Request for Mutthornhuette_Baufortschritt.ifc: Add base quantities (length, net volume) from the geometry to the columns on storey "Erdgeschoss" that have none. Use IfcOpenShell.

First a look at what the model holds.

```python
import ifcopenshell
import ifcopenshell.util.element
import ifcopenshell.util.unit

model = ifcopenshell.open("Mutthornhuette_Baufortschritt.ifc")
print(model.schema)
for unit_type in ("LENGTHUNIT", "AREAUNIT", "VOLUMEUNIT"):
    print(unit_type, ifcopenshell.util.unit.calculate_unit_scale(model, unit_type))
storey = next(s for s in model.by_type("IfcBuildingStorey") if s.Name == "Erdgeschoss")
columns = [e for e in ifcopenshell.util.element.get_decomposition(storey) if e.is_a("IfcColumn")]
for e in sorted(columns, key=lambda e: e.id()):
    print(e.id(), e.is_a(), e.Name, list(ifcopenshell.util.element.get_psets(e, qtos_only=True)), sep=" | ")
```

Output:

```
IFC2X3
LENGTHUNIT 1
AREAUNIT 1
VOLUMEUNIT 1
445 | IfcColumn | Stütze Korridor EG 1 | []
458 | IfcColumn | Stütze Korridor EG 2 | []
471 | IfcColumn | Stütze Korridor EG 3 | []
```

```python
import ifcopenshell
import ifcopenshell.api.pset
import ifcopenshell.geom
import ifcopenshell.util.element
import ifcopenshell.util.shape
import ifcopenshell.util.unit

model = ifcopenshell.open("Mutthornhuette_Baufortschritt.ifc")
unit_scale = ifcopenshell.util.unit.calculate_unit_scale(model)
volume_scale = ifcopenshell.util.unit.calculate_unit_scale(model, "VOLUMEUNIT")
settings = ifcopenshell.geom.settings()

storey = next(s for s in model.by_type("IfcBuildingStorey") if s.Name == "Erdgeschoss")
columns = [e for e in ifcopenshell.util.element.get_decomposition(storey) if e.is_a("IfcColumn")]

for e in sorted(columns, key=lambda e: e.id()):
    if ifcopenshell.util.element.get_psets(e, qtos_only=True, should_inherit=False):
        continue
    # Geometry comes back in metres, in the element's own axes.
    shape = ifcopenshell.geom.create_shape(settings, e)
    values = {
        "Length": ifcopenshell.util.shape.get_z(shape.geometry) / unit_scale,
        "NetVolume": ifcopenshell.util.shape.get_volume(shape.geometry) / volume_scale,
    }
    qto = ifcopenshell.api.pset.add_qto(model, product=e, name="BaseQuantities")
    ifcopenshell.api.pset.edit_qto(model, qto=qto, properties=values)
    print(e.id(), {k: round(v, 3) for k, v in values.items()})

model.write("Mutthornhuette_Baufortschritt_v2.ifc")
```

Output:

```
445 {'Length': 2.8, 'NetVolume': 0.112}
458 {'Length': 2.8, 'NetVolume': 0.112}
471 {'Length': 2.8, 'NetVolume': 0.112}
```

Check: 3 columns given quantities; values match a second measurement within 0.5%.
